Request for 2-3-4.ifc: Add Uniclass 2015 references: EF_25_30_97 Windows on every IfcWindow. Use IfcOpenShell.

First a look at what the model holds.

```python
import ifcopenshell

model = ifcopenshell.open("2-3-4.ifc")
print(model.schema)
print("classifications:", [c.Name for c in model.by_type("IfcClassification")])
for ifc_class in ("IfcDoor", "IfcRoof", "IfcStair", "IfcWall", "IfcWindow"):
    print(ifc_class, len(model.by_type(ifc_class)))
```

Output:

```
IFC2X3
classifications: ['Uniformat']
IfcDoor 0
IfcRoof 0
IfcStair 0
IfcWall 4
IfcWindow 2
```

```python
import ifcopenshell
import ifcopenshell.api.classification

model = ifcopenshell.open("2-3-4.ifc")

# IFC2X3 requires Source and Edition and has no link from the project to the system.
system = model.create_entity("IfcClassification", Source="NBS", Edition="2015", Name="Uniclass 2015")

codes = {
    "IfcWindow": ("EF_25_30_97", "Windows"),
}
for ifc_class, (code, name) in codes.items():
    products = model.by_type(ifc_class)
    ifcopenshell.api.classification.add_reference(
        model, products=products, classification=system, identification=code, name=name
    )
    print(code, len(products))

model.write("2-3-4_updated.ifc")
```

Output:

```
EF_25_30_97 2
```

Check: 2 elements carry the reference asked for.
